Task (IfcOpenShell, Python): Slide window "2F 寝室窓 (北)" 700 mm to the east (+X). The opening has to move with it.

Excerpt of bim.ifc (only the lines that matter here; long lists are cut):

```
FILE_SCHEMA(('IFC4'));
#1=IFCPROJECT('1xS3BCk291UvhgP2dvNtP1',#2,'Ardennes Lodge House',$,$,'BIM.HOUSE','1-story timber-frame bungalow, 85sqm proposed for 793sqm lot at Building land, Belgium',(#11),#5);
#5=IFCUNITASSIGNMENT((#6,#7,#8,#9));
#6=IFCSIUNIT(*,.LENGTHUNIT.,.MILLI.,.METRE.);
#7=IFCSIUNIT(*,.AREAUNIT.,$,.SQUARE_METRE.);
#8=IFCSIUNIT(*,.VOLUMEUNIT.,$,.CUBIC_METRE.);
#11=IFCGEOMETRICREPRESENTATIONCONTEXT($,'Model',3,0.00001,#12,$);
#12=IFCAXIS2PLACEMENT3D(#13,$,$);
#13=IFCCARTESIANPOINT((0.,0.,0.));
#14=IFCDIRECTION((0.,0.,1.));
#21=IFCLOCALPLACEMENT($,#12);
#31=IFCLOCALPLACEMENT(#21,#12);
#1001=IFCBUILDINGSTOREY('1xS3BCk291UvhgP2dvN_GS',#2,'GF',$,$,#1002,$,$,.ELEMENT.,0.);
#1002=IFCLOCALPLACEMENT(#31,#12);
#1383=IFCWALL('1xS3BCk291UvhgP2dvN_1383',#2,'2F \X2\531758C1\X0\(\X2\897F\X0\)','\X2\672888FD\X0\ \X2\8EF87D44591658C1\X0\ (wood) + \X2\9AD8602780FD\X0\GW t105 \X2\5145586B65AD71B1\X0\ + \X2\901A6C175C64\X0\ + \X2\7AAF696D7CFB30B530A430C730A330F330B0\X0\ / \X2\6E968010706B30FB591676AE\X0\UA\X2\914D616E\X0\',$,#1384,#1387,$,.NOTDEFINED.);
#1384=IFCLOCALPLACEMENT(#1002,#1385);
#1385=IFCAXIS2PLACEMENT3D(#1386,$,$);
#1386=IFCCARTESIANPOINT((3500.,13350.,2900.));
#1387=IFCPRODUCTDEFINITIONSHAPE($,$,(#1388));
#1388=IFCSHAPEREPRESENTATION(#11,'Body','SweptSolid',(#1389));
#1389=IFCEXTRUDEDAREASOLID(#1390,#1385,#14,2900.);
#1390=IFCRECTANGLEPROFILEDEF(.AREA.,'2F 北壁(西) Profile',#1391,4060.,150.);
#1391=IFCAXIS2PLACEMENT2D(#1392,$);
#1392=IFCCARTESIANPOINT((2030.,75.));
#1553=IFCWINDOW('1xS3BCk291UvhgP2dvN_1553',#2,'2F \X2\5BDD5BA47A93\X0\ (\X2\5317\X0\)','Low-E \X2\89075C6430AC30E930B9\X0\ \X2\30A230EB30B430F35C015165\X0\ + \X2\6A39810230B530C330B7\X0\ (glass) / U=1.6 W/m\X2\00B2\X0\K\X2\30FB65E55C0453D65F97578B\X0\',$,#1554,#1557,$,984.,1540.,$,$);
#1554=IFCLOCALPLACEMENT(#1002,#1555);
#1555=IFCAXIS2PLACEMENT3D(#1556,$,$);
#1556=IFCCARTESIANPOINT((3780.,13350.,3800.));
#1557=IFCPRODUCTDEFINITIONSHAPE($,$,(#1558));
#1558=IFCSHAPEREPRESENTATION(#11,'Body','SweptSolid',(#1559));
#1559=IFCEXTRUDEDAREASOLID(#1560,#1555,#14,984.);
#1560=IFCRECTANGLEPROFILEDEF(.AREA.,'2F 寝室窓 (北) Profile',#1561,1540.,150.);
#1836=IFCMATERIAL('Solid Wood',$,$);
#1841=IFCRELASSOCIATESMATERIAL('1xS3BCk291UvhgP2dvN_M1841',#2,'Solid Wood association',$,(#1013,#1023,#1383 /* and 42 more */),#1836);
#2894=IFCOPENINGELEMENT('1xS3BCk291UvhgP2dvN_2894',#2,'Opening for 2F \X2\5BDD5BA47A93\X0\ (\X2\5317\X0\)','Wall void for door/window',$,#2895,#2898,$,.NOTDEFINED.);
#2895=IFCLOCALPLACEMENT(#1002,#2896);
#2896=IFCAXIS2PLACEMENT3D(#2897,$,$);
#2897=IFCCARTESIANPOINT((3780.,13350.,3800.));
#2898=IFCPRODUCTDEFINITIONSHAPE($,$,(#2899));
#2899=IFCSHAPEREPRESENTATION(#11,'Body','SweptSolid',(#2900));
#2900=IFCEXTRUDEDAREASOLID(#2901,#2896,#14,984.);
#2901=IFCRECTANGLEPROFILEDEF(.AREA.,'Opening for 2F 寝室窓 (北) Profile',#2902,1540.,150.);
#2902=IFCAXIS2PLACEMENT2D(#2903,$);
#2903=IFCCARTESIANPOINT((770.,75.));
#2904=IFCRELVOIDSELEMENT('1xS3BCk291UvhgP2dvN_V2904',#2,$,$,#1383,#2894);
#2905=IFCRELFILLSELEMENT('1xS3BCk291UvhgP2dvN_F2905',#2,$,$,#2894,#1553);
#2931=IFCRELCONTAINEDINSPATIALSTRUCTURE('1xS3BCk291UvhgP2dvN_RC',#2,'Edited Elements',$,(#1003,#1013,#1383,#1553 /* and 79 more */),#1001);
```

```python
import ifcopenshell
import ifcopenshell.api.geometry
import ifcopenshell.util.placement
import ifcopenshell.util.unit

model = ifcopenshell.open("bim.ifc")
unit_scale = ifcopenshell.util.unit.calculate_unit_scale(model)

window = model.by_guid("1xS3BCk291UvhgP2dvN_1553")
opening = window.FillsVoids[0].RelatingOpeningElement
wall = opening.VoidsElements[0].RelatingBuildingElement

wall_matrix = ifcopenshell.util.placement.get_local_placement(wall.ObjectPlacement)
shift = wall_matrix[:3, 0] * 0.7 / unit_scale
before = ifcopenshell.util.placement.get_local_placement(window.ObjectPlacement)[:3, 3].copy()

# The window is not placed relative to its opening, so move both.
for product in (opening, window):
    matrix = ifcopenshell.util.placement.get_local_placement(product.ObjectPlacement)
    matrix[:3, 3] += shift
    ifcopenshell.api.geometry.edit_object_placement(model, product=product, matrix=matrix, is_si=False)

after = ifcopenshell.util.placement.get_local_placement(window.ObjectPlacement)[:3, 3]
print("window moved by", (after - before).round(3) + 0.0)

model.write("bim-out.ifc")
```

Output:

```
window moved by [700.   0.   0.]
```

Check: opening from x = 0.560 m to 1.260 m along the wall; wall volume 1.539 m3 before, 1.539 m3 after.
